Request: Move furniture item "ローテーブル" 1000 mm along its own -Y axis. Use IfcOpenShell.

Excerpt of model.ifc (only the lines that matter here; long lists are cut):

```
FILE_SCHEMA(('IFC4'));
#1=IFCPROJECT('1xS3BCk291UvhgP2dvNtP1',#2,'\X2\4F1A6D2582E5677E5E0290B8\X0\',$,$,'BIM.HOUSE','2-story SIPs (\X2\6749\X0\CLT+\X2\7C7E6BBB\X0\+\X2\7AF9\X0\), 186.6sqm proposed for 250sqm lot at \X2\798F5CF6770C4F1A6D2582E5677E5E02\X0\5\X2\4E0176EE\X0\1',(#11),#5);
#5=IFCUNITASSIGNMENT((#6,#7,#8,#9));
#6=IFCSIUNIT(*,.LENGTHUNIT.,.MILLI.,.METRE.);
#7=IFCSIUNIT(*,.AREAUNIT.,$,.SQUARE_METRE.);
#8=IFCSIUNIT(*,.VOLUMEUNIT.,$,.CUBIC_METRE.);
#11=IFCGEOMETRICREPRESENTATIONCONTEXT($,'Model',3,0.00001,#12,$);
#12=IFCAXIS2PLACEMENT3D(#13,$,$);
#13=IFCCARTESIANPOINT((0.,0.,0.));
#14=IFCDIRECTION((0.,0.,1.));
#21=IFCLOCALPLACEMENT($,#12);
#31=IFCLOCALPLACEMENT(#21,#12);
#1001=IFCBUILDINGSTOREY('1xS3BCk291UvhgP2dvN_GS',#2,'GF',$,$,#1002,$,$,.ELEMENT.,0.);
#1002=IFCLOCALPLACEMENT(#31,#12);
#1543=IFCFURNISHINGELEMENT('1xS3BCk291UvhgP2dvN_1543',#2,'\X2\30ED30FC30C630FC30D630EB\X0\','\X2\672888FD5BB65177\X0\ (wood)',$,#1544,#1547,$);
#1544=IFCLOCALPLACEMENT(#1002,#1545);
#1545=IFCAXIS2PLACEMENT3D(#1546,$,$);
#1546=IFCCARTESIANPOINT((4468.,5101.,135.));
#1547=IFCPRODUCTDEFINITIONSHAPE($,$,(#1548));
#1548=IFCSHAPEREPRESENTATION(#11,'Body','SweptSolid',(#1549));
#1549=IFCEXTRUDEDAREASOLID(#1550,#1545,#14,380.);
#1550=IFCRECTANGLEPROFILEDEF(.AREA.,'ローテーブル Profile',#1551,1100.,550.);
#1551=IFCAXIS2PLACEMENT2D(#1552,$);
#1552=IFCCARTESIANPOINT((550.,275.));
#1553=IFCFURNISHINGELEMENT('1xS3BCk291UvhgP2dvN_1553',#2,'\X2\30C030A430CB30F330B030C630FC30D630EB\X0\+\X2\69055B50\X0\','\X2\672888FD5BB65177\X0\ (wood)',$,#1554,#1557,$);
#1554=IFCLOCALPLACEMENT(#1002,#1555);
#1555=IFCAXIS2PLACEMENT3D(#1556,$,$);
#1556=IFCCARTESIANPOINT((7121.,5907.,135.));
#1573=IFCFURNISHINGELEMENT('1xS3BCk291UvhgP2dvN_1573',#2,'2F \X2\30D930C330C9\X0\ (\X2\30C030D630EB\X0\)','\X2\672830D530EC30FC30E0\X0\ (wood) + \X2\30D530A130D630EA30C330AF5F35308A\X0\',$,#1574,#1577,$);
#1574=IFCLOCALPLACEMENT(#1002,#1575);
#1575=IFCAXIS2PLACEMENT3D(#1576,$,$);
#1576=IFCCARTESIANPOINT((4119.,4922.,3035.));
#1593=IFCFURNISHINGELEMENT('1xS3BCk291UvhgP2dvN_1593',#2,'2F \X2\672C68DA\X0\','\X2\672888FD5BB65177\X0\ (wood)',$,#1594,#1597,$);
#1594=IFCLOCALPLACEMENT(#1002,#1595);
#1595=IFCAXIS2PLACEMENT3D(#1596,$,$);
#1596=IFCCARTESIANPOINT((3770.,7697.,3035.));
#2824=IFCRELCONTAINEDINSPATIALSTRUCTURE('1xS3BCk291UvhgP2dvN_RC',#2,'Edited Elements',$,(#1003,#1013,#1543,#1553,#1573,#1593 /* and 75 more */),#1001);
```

```python
import ifcopenshell
import ifcopenshell.api.geometry
import ifcopenshell.util.placement
import ifcopenshell.util.unit

model = ifcopenshell.open("model.ifc")
unit_scale = ifcopenshell.util.unit.calculate_unit_scale(model)

item = model.by_id(1543)
matrix = ifcopenshell.util.placement.get_local_placement(item.ObjectPlacement)
matrix[:3, 3] -= matrix[:3, 1] * 1 / unit_scale
ifcopenshell.api.geometry.edit_object_placement(model, product=item, matrix=matrix, is_si=False)

print(ifcopenshell.util.placement.get_local_placement(item.ObjectPlacement).round(3) + 0.0)

model.write("model-out.ifc")
```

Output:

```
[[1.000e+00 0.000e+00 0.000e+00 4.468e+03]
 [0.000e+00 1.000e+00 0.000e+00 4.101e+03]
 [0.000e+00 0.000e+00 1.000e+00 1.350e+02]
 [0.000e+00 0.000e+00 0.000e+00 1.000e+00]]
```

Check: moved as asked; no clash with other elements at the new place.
